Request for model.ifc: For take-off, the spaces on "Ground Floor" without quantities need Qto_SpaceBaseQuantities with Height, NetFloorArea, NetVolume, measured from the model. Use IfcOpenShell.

First a look at what the model holds.

```python
import ifcopenshell
import ifcopenshell.util.element
import ifcopenshell.util.unit

model = ifcopenshell.open("model.ifc")
print(model.schema)
for unit_type in ("LENGTHUNIT", "AREAUNIT", "VOLUMEUNIT"):
    print(unit_type, ifcopenshell.util.unit.calculate_unit_scale(model, unit_type))
storey = next(s for s in model.by_type("IfcBuildingStorey") if s.Name == "Ground Floor")
spaces = [e for e in ifcopenshell.util.element.get_decomposition(storey) if e.is_a("IfcSpace")]
for e in sorted(spaces, key=lambda e: e.id()):
    print(e.id(), e.is_a(), e.Name, list(ifcopenshell.util.element.get_psets(e, qtos_only=True)), sep=" | ")
```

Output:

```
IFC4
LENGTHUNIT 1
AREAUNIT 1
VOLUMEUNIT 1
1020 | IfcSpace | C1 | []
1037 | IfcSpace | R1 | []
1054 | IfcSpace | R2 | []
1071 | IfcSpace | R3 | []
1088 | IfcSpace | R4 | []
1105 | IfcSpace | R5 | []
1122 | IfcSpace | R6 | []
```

```python
import ifcopenshell
import ifcopenshell.api.pset
import ifcopenshell.geom
import ifcopenshell.util.element
import ifcopenshell.util.shape
import ifcopenshell.util.unit

model = ifcopenshell.open("model.ifc")
unit_scale = ifcopenshell.util.unit.calculate_unit_scale(model)
area_scale = ifcopenshell.util.unit.calculate_unit_scale(model, "AREAUNIT")
volume_scale = ifcopenshell.util.unit.calculate_unit_scale(model, "VOLUMEUNIT")
settings = ifcopenshell.geom.settings()

storey = next(s for s in model.by_type("IfcBuildingStorey") if s.Name == "Ground Floor")
spaces = [e for e in ifcopenshell.util.element.get_decomposition(storey) if e.is_a("IfcSpace")]

for e in sorted(spaces, key=lambda e: e.id()):
    if ifcopenshell.util.element.get_psets(e, qtos_only=True, should_inherit=False):
        continue
    # Geometry comes back in metres, in the element's own axes.
    shape = ifcopenshell.geom.create_shape(settings, e)
    values = {
        "Height": ifcopenshell.util.shape.get_z(shape.geometry) / unit_scale,
        "NetFloorArea": ifcopenshell.util.shape.get_footprint_area(shape.geometry) / area_scale,
        "NetVolume": ifcopenshell.util.shape.get_volume(shape.geometry) / volume_scale,
    }
    qto = ifcopenshell.api.pset.add_qto(model, product=e, name="Qto_SpaceBaseQuantities")
    ifcopenshell.api.pset.edit_qto(model, qto=qto, properties=values)
    print(e.id(), {k: round(v, 3) for k, v in values.items()})

model.write("model_v2.ifc")
```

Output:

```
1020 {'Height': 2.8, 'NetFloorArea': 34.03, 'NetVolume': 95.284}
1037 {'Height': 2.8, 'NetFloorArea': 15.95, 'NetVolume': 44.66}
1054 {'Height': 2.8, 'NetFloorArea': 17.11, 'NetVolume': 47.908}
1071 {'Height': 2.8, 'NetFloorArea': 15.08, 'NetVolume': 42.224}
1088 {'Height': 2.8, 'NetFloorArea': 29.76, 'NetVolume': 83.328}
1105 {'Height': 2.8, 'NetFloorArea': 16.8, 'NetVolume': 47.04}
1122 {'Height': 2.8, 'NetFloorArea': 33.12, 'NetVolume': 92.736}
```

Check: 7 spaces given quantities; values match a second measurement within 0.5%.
